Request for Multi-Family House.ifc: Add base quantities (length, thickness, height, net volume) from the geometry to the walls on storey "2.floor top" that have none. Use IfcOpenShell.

First a look at what the model holds.

```python
import ifcopenshell
import ifcopenshell.util.element
import ifcopenshell.util.unit

model = ifcopenshell.open("Multi-Family House.ifc")
print(model.schema)
for unit_type in ("LENGTHUNIT", "AREAUNIT", "VOLUMEUNIT"):
    print(unit_type, ifcopenshell.util.unit.calculate_unit_scale(model, unit_type))
storey = next(s for s in model.by_type("IfcBuildingStorey") if s.Name == "2.floor top")
walls = [e for e in ifcopenshell.util.element.get_decomposition(storey) if e.is_a("IfcWall")]
for e in sorted(walls, key=lambda e: e.id()):
    print(e.id(), e.is_a(), e.Name, list(ifcopenshell.util.element.get_psets(e, qtos_only=True)), sep=" | ")
```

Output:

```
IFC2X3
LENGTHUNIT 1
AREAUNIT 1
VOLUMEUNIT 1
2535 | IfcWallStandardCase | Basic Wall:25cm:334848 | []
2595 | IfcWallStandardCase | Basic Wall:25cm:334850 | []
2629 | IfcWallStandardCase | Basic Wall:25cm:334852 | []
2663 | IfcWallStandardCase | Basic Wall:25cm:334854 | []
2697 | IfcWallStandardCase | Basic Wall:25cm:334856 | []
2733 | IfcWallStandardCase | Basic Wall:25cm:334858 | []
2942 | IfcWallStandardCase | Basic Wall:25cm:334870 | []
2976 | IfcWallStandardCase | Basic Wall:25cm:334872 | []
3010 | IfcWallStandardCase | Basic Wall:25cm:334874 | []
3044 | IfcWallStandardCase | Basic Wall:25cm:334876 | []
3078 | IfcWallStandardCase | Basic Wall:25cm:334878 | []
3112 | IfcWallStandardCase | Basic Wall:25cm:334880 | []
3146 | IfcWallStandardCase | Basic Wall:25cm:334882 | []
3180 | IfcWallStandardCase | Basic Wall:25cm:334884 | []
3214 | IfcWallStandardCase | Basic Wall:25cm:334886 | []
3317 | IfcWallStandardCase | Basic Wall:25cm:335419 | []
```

```python
import ifcopenshell
import ifcopenshell.api.pset
import ifcopenshell.geom
import ifcopenshell.util.element
import ifcopenshell.util.shape
import ifcopenshell.util.unit

model = ifcopenshell.open("Multi-Family House.ifc")
unit_scale = ifcopenshell.util.unit.calculate_unit_scale(model)
volume_scale = ifcopenshell.util.unit.calculate_unit_scale(model, "VOLUMEUNIT")
settings = ifcopenshell.geom.settings()

storey = next(s for s in model.by_type("IfcBuildingStorey") if s.Name == "2.floor top")
walls = [e for e in ifcopenshell.util.element.get_decomposition(storey) if e.is_a("IfcWall")]

for e in sorted(walls, key=lambda e: e.id()):
    if ifcopenshell.util.element.get_psets(e, qtos_only=True, should_inherit=False):
        continue
    # Geometry comes back in metres, in the element's own axes.
    shape = ifcopenshell.geom.create_shape(settings, e)
    values = {
        "Length": ifcopenshell.util.shape.get_x(shape.geometry) / unit_scale,
        "Width": ifcopenshell.util.shape.get_y(shape.geometry) / unit_scale,
        "Height": ifcopenshell.util.shape.get_z(shape.geometry) / unit_scale,
        "NetVolume": ifcopenshell.util.shape.get_volume(shape.geometry) / volume_scale,
    }
    qto = ifcopenshell.api.pset.add_qto(model, product=e, name="BaseQuantities")
    ifcopenshell.api.pset.edit_qto(model, qto=qto, properties=values)
    print(e.id(), {k: round(v, 3) for k, v in values.items()})

model.write("Multi-Family House-out.ifc")
```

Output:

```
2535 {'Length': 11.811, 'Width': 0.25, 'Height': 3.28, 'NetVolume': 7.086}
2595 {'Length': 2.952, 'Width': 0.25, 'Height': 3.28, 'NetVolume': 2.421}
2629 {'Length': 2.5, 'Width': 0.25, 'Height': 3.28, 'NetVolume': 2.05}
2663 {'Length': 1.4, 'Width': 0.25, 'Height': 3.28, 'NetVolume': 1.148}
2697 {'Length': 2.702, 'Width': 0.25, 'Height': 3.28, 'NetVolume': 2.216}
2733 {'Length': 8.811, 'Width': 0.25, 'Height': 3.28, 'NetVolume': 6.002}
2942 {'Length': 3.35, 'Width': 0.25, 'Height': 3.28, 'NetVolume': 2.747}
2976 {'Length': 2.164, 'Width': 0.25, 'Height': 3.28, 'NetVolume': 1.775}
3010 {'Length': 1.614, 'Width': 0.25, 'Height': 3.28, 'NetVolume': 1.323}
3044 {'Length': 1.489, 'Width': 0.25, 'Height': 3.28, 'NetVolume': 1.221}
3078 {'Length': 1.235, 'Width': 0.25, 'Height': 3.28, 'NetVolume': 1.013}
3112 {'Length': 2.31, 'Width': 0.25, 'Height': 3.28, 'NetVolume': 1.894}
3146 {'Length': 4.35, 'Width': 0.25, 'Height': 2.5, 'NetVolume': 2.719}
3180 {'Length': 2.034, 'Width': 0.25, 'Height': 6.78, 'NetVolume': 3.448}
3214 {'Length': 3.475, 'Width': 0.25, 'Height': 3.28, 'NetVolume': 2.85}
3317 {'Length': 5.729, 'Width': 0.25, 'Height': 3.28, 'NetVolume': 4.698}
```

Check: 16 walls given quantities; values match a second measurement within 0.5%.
